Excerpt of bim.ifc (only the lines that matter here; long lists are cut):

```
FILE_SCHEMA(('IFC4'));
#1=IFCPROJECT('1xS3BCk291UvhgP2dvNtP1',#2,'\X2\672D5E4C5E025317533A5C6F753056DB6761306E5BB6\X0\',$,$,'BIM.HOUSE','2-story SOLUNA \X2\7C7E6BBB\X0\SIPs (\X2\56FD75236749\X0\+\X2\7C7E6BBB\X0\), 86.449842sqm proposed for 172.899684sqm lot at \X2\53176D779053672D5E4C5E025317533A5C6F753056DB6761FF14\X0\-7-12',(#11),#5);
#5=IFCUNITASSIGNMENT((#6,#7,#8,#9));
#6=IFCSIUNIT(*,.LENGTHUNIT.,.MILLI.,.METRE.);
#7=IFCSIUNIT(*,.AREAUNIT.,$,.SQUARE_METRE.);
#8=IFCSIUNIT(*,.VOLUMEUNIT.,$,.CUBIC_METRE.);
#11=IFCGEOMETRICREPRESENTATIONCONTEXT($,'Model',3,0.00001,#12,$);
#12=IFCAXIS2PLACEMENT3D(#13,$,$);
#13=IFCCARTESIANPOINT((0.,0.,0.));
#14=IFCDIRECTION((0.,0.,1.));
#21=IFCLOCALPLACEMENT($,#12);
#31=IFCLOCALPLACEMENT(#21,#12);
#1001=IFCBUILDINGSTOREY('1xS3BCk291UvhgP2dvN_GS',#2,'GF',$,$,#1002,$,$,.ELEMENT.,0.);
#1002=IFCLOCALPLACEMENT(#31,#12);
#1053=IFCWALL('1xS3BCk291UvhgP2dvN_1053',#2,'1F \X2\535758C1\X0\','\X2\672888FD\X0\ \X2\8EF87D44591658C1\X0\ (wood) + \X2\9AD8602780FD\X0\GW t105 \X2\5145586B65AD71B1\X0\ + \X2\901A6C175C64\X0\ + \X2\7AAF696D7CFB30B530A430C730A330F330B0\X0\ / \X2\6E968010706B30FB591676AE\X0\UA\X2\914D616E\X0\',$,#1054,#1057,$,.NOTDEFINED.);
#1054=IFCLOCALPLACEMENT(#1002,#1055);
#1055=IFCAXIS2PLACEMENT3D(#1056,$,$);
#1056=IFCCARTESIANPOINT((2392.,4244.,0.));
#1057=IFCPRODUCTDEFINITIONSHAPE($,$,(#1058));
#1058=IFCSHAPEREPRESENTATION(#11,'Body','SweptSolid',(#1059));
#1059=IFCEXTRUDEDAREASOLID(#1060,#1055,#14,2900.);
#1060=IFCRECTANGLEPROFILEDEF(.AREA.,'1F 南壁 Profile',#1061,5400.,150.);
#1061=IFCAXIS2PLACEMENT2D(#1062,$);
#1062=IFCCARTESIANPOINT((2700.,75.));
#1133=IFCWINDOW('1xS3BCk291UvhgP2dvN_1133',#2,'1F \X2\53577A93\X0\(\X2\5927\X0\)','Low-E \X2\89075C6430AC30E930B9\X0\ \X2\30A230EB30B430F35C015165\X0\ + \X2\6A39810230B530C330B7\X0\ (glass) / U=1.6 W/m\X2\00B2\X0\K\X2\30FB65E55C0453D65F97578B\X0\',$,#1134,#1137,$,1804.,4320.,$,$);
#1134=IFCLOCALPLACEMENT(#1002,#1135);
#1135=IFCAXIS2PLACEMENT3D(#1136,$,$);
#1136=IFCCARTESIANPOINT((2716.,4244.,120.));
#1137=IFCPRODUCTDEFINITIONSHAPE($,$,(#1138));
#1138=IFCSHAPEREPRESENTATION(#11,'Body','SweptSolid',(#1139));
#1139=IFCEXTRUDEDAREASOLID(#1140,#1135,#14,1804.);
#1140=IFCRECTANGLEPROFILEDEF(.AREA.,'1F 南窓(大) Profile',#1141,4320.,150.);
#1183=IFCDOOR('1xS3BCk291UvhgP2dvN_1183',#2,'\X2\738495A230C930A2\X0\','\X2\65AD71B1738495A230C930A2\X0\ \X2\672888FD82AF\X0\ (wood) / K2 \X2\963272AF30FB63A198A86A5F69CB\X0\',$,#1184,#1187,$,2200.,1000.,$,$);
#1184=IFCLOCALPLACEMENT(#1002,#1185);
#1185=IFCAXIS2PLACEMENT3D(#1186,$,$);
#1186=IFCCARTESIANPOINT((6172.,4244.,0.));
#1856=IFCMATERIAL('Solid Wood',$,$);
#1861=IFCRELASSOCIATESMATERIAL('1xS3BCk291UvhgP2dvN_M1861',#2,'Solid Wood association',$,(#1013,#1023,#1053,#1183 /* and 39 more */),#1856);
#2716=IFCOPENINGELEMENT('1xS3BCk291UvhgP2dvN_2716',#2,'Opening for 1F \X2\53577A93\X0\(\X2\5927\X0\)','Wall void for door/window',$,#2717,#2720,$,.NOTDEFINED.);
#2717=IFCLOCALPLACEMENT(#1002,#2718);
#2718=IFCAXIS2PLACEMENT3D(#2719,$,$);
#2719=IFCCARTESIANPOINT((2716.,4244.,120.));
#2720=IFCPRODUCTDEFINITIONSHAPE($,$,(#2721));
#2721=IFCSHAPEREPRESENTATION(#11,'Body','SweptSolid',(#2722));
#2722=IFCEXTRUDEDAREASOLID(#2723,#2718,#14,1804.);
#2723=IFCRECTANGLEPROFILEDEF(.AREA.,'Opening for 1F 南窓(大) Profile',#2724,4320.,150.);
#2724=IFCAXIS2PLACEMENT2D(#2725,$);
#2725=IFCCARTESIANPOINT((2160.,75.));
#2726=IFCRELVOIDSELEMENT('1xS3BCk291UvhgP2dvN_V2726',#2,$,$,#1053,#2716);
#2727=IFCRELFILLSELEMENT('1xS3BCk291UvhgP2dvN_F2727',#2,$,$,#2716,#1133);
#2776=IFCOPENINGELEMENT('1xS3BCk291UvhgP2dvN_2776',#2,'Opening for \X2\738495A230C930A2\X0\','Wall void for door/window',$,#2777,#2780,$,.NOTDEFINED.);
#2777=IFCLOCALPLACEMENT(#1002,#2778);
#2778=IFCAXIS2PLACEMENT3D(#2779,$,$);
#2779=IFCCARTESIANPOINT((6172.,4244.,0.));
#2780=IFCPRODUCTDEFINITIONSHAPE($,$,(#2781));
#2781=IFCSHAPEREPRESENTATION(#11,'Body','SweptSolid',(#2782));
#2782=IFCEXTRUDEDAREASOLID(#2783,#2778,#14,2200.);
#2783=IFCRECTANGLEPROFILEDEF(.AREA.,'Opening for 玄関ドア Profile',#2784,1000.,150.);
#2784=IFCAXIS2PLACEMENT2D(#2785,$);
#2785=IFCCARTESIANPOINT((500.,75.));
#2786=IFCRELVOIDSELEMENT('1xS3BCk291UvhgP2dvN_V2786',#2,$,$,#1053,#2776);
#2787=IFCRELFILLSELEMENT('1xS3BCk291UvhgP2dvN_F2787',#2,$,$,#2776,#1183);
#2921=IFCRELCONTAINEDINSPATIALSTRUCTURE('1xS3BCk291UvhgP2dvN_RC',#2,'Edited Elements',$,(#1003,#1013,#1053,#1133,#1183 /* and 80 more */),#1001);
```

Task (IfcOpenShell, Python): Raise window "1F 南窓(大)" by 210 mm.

```python
import numpy as np
import ifcopenshell
import ifcopenshell.api.geometry
import ifcopenshell.util.placement
import ifcopenshell.util.unit

model = ifcopenshell.open("bim.ifc")
unit_scale = ifcopenshell.util.unit.calculate_unit_scale(model)

window = model.by_guid("1xS3BCk291UvhgP2dvN_1133")
opening = window.FillsVoids[0].RelatingOpeningElement
dz = 210.0

shift = np.array([0.0, 0.0, dz])
# The window is not placed relative to its opening, so move both.
for product in (opening, window):
    matrix = ifcopenshell.util.placement.get_local_placement(product.ObjectPlacement)
    matrix[:3, 3] += shift
    ifcopenshell.api.geometry.edit_object_placement(model, product=product, matrix=matrix, is_si=False)

print(f"moved by {dz * unit_scale:+.3f} m")

model.write("bim_updated.ifc")
```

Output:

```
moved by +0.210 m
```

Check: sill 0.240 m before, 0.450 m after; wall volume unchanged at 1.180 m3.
